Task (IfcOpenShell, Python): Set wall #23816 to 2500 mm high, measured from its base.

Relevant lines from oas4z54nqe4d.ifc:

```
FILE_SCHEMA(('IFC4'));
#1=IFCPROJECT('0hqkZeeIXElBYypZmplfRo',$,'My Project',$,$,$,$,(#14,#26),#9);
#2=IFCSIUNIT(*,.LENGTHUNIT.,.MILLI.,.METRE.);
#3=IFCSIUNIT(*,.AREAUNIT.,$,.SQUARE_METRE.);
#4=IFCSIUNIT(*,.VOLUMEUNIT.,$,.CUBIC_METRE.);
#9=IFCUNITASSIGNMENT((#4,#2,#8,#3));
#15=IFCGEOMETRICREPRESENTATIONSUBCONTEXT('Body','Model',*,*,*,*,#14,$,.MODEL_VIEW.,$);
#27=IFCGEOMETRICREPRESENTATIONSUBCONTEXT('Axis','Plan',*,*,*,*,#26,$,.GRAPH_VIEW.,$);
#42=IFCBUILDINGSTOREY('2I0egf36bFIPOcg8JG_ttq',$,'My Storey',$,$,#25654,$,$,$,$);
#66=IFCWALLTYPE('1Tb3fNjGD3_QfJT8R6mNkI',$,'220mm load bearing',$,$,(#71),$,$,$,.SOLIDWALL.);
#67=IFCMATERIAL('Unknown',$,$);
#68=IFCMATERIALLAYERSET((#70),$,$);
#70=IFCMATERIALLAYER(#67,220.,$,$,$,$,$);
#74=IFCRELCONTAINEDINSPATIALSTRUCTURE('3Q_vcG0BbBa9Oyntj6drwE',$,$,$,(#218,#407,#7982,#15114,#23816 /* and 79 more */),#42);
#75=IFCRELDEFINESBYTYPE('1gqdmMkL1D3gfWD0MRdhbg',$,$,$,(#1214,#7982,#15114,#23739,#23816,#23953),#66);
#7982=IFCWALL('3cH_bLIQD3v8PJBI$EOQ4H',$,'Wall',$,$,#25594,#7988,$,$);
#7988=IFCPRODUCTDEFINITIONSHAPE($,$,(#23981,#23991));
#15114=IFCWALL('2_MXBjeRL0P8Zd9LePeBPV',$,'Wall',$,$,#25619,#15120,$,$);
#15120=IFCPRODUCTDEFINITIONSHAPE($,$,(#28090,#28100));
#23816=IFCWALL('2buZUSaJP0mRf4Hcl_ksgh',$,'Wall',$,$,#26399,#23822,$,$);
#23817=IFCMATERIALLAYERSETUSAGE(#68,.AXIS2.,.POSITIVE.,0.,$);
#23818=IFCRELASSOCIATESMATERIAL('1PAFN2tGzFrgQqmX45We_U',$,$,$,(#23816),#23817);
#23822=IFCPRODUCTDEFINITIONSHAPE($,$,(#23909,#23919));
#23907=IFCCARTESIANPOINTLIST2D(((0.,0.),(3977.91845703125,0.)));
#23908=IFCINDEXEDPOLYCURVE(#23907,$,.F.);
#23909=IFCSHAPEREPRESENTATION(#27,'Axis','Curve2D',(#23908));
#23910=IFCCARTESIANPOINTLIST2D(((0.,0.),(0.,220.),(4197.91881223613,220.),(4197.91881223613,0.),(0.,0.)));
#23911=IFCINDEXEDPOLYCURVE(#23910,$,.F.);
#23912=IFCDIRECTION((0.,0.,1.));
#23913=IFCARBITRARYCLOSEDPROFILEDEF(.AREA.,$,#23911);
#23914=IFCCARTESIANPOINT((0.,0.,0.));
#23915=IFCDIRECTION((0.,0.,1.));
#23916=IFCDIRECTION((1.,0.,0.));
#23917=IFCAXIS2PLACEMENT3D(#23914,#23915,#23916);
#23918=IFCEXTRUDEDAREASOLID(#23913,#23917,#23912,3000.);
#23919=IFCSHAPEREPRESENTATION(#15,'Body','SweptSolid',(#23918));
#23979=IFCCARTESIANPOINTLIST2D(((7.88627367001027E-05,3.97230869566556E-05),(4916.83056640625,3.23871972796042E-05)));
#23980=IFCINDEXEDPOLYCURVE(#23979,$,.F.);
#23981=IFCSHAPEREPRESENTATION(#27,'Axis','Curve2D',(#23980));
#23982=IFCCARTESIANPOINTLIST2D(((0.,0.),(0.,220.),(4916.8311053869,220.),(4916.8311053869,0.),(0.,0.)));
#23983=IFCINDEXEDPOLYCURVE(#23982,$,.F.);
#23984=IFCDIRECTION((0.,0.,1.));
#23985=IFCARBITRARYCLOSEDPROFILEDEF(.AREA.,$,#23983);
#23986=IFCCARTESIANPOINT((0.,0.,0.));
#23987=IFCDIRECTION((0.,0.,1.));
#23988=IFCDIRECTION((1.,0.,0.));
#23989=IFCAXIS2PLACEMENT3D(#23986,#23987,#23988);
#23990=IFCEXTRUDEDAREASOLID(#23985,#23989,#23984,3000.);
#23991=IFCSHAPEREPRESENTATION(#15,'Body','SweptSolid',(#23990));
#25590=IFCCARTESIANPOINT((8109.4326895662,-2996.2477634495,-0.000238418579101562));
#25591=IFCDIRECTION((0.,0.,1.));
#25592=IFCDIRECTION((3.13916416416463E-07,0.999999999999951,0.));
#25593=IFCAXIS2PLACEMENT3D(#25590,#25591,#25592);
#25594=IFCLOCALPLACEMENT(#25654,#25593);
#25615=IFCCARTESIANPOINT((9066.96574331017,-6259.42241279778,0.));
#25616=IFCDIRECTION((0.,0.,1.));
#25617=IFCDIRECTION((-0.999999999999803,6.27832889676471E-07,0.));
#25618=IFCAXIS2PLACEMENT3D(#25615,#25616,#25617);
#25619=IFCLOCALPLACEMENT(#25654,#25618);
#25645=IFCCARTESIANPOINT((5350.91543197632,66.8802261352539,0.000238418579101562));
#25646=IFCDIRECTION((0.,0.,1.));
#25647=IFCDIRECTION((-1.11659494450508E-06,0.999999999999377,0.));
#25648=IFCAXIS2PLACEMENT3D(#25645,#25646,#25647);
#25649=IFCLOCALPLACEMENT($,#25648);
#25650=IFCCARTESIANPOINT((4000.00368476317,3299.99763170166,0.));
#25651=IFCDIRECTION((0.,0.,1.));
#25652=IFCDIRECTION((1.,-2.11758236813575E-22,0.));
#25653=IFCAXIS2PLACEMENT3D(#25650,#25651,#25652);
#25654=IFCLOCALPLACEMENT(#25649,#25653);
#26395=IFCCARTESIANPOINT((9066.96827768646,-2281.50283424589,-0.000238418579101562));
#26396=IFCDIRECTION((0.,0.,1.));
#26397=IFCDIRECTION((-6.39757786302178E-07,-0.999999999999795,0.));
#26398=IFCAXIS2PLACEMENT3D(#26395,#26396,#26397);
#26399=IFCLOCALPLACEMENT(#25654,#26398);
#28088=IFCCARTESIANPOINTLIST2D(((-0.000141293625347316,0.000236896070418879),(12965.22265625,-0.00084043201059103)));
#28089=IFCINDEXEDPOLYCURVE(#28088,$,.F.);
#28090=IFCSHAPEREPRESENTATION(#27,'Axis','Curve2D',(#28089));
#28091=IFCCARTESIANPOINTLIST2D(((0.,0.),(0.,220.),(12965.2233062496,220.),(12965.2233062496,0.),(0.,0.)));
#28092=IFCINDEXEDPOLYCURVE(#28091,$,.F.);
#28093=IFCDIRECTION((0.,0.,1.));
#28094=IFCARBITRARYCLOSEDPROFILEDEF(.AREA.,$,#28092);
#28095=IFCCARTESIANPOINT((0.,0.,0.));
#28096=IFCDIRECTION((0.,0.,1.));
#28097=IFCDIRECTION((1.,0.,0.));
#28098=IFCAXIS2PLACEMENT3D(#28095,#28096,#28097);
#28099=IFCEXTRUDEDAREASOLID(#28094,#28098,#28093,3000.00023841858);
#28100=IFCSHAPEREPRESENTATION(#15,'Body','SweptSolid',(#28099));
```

```python
import ifcopenshell
import ifcopenshell.geom
import ifcopenshell.util.representation
import ifcopenshell.util.shape
import ifcopenshell.util.unit

model = ifcopenshell.open("oas4z54nqe4d.ifc")
unit_scale = ifcopenshell.util.unit.calculate_unit_scale(model)
settings = ifcopenshell.geom.settings()


def volume(element):
    """Net volume in cubic metres, openings subtracted."""
    shape = ifcopenshell.geom.create_shape(settings, element)
    return ifcopenshell.util.shape.get_volume(shape.geometry)


wall = model.by_guid("2buZUSaJP0mRf4Hcl_ksgh")
before = volume(wall)

body = ifcopenshell.util.representation.get_representation(wall, "Model", "Body")
solid = body.Items[0]
old_height = solid.Depth
solid.Depth = 2.5 / unit_scale
after = volume(wall)

print(f"height {old_height:g} -> {solid.Depth:g}, volume {before:.3f} -> {after:.3f} m3")

model.write("oas4z54nqe4d-out.ifc")
```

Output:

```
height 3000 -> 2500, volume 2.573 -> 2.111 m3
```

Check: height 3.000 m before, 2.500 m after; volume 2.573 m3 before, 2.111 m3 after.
